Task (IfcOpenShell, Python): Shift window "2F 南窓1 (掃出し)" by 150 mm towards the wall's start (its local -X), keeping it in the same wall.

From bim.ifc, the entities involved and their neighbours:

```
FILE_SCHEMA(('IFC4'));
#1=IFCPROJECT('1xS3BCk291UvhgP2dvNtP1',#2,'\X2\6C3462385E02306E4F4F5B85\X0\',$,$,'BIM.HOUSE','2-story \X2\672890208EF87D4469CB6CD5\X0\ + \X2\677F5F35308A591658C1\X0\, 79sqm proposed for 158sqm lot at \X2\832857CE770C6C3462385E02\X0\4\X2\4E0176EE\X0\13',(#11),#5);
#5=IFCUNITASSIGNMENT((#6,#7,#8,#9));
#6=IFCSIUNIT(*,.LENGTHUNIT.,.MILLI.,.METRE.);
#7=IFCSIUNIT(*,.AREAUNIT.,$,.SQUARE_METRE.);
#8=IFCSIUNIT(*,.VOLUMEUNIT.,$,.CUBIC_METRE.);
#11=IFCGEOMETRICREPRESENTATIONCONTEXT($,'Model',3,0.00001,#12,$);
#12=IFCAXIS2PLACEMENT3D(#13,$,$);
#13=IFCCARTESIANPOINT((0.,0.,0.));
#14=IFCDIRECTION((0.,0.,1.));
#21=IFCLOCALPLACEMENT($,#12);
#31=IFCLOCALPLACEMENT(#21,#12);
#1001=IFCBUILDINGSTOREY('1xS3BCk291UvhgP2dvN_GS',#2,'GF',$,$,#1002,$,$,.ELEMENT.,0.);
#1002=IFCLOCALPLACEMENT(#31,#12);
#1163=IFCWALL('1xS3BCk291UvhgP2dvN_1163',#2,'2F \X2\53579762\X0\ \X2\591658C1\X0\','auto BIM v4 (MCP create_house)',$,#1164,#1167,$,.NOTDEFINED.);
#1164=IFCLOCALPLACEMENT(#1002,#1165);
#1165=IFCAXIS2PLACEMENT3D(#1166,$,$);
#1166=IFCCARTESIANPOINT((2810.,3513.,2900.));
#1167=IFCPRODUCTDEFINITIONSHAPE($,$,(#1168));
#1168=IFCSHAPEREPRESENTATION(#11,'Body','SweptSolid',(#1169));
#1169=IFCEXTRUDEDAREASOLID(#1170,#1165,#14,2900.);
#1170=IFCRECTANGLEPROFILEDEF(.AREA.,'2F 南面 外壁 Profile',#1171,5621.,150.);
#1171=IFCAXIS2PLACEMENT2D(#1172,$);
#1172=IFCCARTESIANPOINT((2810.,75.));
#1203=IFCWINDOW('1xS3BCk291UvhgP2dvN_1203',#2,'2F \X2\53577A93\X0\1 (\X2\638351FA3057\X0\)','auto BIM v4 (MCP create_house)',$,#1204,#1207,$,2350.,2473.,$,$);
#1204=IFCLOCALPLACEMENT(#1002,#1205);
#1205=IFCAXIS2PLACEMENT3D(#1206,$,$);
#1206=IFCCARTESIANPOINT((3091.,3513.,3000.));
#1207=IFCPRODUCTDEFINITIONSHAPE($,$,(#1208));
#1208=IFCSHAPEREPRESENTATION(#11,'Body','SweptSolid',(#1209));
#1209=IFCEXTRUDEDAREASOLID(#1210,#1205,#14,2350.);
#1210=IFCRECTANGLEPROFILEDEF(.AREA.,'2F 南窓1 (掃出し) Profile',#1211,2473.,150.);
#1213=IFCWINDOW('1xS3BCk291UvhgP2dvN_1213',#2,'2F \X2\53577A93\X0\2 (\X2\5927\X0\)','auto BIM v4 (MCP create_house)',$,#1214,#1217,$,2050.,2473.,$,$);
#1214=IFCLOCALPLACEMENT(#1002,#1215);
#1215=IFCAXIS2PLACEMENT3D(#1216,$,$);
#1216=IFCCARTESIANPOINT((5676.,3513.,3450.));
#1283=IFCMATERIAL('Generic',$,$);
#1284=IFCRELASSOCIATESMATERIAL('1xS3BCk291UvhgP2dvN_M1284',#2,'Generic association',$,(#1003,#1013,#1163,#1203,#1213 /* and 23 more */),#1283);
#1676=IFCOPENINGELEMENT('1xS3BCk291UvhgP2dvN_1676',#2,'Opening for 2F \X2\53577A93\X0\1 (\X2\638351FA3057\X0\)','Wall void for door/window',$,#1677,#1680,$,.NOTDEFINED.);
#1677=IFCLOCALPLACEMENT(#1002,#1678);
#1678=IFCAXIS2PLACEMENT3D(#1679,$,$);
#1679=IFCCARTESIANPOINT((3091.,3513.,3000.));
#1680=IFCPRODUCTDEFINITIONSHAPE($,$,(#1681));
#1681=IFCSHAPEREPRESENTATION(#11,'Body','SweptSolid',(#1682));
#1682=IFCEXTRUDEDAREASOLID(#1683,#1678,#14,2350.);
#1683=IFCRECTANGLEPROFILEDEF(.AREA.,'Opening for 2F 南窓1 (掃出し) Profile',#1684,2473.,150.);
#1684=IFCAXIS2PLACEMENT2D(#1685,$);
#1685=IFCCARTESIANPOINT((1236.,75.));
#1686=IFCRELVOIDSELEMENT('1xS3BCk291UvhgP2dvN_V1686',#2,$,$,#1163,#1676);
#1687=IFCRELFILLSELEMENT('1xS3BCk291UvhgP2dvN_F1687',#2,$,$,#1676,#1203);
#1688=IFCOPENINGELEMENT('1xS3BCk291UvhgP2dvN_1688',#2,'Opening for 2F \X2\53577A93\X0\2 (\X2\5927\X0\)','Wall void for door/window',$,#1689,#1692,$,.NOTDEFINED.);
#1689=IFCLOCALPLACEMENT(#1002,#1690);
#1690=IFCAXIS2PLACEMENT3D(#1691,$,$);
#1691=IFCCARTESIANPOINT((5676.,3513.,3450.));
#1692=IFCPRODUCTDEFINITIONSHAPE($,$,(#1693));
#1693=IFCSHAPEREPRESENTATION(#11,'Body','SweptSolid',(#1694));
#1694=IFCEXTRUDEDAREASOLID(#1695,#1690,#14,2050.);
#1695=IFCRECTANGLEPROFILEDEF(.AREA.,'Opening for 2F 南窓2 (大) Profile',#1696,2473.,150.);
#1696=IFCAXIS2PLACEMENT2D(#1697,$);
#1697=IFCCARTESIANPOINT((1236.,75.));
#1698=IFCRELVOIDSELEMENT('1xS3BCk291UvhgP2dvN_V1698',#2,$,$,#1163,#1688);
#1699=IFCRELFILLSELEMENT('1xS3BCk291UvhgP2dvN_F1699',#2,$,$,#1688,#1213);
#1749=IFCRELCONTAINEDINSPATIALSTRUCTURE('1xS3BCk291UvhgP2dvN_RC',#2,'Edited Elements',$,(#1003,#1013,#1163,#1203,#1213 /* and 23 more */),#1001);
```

```python
import ifcopenshell
import ifcopenshell.api.geometry
import ifcopenshell.util.placement

model = ifcopenshell.open("bim.ifc")

window = model.by_id(1203)
opening = window.FillsVoids[0].RelatingOpeningElement
wall = opening.VoidsElements[0].RelatingBuildingElement

wall_matrix = ifcopenshell.util.placement.get_local_placement(wall.ObjectPlacement)
shift = wall_matrix[:3, 0] * -150.0
before = ifcopenshell.util.placement.get_local_placement(window.ObjectPlacement)[:3, 3].copy()

# The window is not placed relative to its opening, so move both.
for product in (opening, window):
    matrix = ifcopenshell.util.placement.get_local_placement(product.ObjectPlacement)
    matrix[:3, 3] += shift
    ifcopenshell.api.geometry.edit_object_placement(model, product=product, matrix=matrix, is_si=False)

after = ifcopenshell.util.placement.get_local_placement(window.ObjectPlacement)[:3, 3]
print("window moved by", (after - before).round(3) + 0.0)

model.write("bim_edited.ifc")
```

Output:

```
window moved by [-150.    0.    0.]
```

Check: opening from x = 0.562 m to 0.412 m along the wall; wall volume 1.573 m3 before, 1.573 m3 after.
